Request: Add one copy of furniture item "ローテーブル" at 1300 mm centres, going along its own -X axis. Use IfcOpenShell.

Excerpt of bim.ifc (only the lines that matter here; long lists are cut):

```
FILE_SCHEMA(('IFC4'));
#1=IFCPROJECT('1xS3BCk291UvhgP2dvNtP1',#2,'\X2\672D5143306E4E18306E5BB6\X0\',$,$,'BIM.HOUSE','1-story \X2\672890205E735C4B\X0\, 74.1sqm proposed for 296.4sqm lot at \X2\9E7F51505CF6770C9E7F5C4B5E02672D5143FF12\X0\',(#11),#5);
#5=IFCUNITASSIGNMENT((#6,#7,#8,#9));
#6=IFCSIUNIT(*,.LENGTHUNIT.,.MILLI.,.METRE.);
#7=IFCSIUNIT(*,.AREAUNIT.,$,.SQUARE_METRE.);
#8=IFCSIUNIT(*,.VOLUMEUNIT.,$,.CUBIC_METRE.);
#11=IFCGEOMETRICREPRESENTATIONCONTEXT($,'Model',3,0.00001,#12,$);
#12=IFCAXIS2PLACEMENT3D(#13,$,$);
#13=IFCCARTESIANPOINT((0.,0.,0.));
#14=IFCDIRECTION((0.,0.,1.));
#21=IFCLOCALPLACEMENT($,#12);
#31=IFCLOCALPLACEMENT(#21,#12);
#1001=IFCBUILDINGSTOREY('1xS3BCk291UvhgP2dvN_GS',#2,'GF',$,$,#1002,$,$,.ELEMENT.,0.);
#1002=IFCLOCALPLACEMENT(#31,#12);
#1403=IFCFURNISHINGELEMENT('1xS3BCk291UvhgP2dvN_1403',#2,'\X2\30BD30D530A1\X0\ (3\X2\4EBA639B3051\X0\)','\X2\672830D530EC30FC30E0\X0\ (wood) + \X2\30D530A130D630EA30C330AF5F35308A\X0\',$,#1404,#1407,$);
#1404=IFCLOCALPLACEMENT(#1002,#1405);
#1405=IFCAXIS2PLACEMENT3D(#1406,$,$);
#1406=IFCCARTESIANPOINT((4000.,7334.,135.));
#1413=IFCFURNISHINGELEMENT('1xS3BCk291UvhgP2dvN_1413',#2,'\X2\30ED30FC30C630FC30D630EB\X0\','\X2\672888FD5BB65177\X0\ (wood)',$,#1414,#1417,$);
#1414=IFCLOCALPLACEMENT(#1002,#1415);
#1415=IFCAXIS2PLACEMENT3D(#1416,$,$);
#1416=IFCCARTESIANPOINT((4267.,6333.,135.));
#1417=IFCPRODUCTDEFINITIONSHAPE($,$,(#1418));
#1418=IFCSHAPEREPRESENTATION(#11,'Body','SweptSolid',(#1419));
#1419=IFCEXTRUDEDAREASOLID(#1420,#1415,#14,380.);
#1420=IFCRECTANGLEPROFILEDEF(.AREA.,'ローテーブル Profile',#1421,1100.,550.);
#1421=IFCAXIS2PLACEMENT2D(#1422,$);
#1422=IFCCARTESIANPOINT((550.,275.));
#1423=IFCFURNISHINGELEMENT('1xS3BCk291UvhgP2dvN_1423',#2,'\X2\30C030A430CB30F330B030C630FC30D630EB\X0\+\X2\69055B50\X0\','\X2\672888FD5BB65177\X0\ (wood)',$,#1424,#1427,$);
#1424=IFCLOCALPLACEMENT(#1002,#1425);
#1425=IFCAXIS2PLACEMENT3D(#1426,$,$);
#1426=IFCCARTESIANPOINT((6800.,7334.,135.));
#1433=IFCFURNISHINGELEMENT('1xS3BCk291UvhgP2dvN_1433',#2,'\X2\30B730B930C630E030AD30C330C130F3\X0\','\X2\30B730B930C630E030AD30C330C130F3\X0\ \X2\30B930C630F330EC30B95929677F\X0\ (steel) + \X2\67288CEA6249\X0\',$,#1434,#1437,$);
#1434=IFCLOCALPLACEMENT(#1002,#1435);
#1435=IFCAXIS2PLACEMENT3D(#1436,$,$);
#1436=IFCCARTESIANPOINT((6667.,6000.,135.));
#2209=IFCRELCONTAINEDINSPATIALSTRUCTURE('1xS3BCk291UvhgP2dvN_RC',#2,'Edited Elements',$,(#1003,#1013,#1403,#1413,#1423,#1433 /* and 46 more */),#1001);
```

```python
import ifcopenshell
import ifcopenshell.api.geometry
import ifcopenshell.api.root
import ifcopenshell.util.element
import ifcopenshell.util.placement

model = ifcopenshell.open("bim.ifc")


def reuse_history(source, copy):
    """copy_class also copies each property set's owner history, people and application; keep the originals."""
    for rel in copy.IsDefinedBy:
        if rel.is_a("IfcRelDefinesByProperties") and (history := rel.RelatingPropertyDefinition.OwnerHistory):
            rel.RelatingPropertyDefinition.OwnerHistory = source.OwnerHistory
            ifcopenshell.util.element.remove_deep2(model, history)


source = model.by_guid("1xS3BCk291UvhgP2dvN_1413")
base = ifcopenshell.util.placement.get_local_placement(source.ObjectPlacement)
step = -base[:3, 0] * 1300.0

for i in range(1, 2):
    copy = ifcopenshell.api.root.copy_class(model, product=source)
    copy.Representation = ifcopenshell.util.element.copy_deep(
        model, source.Representation, exclude=["IfcGeometricRepresentationContext", "IfcRepresentationMap"]
    )
    reuse_history(source, copy)
    matrix = base.copy()
    matrix[:3, 3] += i * step
    print("added at", matrix[:3, 3].round(3) + 0.0)
    ifcopenshell.api.geometry.edit_object_placement(model, product=copy, matrix=matrix, is_si=False)

model.write("bim_v2.ifc")
```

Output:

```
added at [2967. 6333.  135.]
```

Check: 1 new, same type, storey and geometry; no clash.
